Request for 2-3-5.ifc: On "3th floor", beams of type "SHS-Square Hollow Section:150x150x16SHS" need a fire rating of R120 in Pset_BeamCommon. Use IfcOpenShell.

First a look at what the model holds.

```python
import ifcopenshell
import ifcopenshell.util.element

model = ifcopenshell.open("2-3-5.ifc")
print(model.schema)
storey = next(s for s in model.by_type("IfcBuildingStorey") if s.Name == "3th floor")
beams = [e for e in ifcopenshell.util.element.get_decomposition(storey) if e.is_a("IfcBeam")]
seen = {}
for e in beams:
    element_type = ifcopenshell.util.element.get_type(e)
    key = (element_type.Name if element_type != e and element_type else None, ifcopenshell.util.element.get_pset(e, "Pset_BeamCommon", "FireRating"))
    seen[key] = seen.get(key, 0) + 1
for (name, value), count in sorted(seen.items(), key=str):
    print(count, "x", name, "|", value)
```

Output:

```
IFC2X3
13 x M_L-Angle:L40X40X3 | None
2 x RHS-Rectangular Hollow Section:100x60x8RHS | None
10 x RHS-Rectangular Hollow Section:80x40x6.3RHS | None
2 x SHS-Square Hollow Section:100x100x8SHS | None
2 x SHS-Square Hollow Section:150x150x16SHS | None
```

```python
import ifcopenshell
import ifcopenshell.api.pset
import ifcopenshell.util.element

model = ifcopenshell.open("2-3-5.ifc")

storey = next(s for s in model.by_type("IfcBuildingStorey") if s.Name == "3th floor")
beams = [e for e in ifcopenshell.util.element.get_decomposition(storey) if e.is_a("IfcBeam")]

count = 0
for e in beams:
    element_type = ifcopenshell.util.element.get_type(e)
    if element_type in (None, e) or element_type.Name != "SHS-Square Hollow Section:150x150x16SHS":
        continue
    # add_pset returns the element's existing set when there is one.
    pset = ifcopenshell.api.pset.add_pset(model, product=e, name="Pset_BeamCommon")
    ifcopenshell.api.pset.edit_pset(model, pset=pset, properties={"FireRating": "R120"})
    count += 1

print(count, "beams updated")

model.write("2-3-5-out.ifc")
```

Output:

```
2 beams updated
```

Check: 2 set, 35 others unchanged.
